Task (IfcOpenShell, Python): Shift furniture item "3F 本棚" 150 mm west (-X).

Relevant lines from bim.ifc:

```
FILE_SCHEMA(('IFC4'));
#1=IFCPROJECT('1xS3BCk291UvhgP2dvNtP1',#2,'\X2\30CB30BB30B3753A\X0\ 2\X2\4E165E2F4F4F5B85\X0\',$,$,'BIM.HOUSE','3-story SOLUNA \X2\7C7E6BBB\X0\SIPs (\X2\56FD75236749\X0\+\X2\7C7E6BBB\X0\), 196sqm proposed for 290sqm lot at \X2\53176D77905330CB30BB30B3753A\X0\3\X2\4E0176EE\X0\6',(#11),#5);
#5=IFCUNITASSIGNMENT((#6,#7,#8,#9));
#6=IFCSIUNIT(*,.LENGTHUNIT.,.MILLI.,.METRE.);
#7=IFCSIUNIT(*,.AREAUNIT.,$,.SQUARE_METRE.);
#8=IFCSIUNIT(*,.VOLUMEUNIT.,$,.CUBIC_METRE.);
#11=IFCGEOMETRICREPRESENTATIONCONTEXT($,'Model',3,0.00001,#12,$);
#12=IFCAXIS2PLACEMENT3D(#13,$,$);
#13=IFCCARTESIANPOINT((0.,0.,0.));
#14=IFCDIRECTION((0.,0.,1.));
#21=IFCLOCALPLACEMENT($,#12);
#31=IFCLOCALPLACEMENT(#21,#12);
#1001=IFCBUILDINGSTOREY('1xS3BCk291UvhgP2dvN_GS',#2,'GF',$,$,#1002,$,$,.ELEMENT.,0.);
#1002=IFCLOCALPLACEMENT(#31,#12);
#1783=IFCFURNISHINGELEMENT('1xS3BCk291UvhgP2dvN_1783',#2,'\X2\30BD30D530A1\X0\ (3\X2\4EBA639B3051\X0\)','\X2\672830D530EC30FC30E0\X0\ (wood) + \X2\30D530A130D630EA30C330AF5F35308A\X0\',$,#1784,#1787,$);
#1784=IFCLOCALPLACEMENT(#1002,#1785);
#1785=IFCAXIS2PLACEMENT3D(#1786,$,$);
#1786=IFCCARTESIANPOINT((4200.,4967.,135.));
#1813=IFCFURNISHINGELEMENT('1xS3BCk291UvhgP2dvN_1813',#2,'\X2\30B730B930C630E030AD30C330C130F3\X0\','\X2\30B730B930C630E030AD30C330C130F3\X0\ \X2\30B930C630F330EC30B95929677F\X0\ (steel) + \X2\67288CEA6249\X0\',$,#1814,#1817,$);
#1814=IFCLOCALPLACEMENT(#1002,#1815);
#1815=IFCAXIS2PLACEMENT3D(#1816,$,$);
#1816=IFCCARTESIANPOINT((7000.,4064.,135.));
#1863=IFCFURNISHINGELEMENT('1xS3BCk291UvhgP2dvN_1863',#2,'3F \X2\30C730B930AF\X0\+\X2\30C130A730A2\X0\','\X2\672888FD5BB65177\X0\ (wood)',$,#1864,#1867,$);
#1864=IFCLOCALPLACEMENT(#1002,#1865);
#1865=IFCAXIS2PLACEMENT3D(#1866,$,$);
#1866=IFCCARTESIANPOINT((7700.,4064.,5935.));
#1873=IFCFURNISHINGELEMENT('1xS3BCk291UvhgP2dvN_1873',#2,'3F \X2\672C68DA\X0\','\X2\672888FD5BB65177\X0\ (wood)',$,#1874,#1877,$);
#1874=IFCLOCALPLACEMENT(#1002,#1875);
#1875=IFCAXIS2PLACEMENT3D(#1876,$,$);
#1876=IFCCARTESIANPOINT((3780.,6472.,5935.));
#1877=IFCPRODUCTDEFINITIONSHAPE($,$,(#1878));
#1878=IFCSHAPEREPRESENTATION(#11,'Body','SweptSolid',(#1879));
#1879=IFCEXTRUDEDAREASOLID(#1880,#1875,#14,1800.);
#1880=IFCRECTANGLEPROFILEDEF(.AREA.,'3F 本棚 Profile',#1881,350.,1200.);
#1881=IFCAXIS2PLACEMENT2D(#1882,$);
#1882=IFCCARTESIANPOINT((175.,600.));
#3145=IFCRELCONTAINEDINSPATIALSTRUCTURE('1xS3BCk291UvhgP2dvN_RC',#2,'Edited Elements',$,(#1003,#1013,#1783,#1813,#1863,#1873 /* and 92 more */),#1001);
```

```python
import ifcopenshell
import ifcopenshell.api.geometry
import ifcopenshell.util.placement

model = ifcopenshell.open("bim.ifc")

item = model.by_id(1873)
matrix = ifcopenshell.util.placement.get_local_placement(item.ObjectPlacement)
matrix[0, 3] -= 150.0
ifcopenshell.api.geometry.edit_object_placement(model, product=item, matrix=matrix, is_si=False)

print(ifcopenshell.util.placement.get_local_placement(item.ObjectPlacement).round(3) + 0.0)

model.write("bim_edited.ifc")
```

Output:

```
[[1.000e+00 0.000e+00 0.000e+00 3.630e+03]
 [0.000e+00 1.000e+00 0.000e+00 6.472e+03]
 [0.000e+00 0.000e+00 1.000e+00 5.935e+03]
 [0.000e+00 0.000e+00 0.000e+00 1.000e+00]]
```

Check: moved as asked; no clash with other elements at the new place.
